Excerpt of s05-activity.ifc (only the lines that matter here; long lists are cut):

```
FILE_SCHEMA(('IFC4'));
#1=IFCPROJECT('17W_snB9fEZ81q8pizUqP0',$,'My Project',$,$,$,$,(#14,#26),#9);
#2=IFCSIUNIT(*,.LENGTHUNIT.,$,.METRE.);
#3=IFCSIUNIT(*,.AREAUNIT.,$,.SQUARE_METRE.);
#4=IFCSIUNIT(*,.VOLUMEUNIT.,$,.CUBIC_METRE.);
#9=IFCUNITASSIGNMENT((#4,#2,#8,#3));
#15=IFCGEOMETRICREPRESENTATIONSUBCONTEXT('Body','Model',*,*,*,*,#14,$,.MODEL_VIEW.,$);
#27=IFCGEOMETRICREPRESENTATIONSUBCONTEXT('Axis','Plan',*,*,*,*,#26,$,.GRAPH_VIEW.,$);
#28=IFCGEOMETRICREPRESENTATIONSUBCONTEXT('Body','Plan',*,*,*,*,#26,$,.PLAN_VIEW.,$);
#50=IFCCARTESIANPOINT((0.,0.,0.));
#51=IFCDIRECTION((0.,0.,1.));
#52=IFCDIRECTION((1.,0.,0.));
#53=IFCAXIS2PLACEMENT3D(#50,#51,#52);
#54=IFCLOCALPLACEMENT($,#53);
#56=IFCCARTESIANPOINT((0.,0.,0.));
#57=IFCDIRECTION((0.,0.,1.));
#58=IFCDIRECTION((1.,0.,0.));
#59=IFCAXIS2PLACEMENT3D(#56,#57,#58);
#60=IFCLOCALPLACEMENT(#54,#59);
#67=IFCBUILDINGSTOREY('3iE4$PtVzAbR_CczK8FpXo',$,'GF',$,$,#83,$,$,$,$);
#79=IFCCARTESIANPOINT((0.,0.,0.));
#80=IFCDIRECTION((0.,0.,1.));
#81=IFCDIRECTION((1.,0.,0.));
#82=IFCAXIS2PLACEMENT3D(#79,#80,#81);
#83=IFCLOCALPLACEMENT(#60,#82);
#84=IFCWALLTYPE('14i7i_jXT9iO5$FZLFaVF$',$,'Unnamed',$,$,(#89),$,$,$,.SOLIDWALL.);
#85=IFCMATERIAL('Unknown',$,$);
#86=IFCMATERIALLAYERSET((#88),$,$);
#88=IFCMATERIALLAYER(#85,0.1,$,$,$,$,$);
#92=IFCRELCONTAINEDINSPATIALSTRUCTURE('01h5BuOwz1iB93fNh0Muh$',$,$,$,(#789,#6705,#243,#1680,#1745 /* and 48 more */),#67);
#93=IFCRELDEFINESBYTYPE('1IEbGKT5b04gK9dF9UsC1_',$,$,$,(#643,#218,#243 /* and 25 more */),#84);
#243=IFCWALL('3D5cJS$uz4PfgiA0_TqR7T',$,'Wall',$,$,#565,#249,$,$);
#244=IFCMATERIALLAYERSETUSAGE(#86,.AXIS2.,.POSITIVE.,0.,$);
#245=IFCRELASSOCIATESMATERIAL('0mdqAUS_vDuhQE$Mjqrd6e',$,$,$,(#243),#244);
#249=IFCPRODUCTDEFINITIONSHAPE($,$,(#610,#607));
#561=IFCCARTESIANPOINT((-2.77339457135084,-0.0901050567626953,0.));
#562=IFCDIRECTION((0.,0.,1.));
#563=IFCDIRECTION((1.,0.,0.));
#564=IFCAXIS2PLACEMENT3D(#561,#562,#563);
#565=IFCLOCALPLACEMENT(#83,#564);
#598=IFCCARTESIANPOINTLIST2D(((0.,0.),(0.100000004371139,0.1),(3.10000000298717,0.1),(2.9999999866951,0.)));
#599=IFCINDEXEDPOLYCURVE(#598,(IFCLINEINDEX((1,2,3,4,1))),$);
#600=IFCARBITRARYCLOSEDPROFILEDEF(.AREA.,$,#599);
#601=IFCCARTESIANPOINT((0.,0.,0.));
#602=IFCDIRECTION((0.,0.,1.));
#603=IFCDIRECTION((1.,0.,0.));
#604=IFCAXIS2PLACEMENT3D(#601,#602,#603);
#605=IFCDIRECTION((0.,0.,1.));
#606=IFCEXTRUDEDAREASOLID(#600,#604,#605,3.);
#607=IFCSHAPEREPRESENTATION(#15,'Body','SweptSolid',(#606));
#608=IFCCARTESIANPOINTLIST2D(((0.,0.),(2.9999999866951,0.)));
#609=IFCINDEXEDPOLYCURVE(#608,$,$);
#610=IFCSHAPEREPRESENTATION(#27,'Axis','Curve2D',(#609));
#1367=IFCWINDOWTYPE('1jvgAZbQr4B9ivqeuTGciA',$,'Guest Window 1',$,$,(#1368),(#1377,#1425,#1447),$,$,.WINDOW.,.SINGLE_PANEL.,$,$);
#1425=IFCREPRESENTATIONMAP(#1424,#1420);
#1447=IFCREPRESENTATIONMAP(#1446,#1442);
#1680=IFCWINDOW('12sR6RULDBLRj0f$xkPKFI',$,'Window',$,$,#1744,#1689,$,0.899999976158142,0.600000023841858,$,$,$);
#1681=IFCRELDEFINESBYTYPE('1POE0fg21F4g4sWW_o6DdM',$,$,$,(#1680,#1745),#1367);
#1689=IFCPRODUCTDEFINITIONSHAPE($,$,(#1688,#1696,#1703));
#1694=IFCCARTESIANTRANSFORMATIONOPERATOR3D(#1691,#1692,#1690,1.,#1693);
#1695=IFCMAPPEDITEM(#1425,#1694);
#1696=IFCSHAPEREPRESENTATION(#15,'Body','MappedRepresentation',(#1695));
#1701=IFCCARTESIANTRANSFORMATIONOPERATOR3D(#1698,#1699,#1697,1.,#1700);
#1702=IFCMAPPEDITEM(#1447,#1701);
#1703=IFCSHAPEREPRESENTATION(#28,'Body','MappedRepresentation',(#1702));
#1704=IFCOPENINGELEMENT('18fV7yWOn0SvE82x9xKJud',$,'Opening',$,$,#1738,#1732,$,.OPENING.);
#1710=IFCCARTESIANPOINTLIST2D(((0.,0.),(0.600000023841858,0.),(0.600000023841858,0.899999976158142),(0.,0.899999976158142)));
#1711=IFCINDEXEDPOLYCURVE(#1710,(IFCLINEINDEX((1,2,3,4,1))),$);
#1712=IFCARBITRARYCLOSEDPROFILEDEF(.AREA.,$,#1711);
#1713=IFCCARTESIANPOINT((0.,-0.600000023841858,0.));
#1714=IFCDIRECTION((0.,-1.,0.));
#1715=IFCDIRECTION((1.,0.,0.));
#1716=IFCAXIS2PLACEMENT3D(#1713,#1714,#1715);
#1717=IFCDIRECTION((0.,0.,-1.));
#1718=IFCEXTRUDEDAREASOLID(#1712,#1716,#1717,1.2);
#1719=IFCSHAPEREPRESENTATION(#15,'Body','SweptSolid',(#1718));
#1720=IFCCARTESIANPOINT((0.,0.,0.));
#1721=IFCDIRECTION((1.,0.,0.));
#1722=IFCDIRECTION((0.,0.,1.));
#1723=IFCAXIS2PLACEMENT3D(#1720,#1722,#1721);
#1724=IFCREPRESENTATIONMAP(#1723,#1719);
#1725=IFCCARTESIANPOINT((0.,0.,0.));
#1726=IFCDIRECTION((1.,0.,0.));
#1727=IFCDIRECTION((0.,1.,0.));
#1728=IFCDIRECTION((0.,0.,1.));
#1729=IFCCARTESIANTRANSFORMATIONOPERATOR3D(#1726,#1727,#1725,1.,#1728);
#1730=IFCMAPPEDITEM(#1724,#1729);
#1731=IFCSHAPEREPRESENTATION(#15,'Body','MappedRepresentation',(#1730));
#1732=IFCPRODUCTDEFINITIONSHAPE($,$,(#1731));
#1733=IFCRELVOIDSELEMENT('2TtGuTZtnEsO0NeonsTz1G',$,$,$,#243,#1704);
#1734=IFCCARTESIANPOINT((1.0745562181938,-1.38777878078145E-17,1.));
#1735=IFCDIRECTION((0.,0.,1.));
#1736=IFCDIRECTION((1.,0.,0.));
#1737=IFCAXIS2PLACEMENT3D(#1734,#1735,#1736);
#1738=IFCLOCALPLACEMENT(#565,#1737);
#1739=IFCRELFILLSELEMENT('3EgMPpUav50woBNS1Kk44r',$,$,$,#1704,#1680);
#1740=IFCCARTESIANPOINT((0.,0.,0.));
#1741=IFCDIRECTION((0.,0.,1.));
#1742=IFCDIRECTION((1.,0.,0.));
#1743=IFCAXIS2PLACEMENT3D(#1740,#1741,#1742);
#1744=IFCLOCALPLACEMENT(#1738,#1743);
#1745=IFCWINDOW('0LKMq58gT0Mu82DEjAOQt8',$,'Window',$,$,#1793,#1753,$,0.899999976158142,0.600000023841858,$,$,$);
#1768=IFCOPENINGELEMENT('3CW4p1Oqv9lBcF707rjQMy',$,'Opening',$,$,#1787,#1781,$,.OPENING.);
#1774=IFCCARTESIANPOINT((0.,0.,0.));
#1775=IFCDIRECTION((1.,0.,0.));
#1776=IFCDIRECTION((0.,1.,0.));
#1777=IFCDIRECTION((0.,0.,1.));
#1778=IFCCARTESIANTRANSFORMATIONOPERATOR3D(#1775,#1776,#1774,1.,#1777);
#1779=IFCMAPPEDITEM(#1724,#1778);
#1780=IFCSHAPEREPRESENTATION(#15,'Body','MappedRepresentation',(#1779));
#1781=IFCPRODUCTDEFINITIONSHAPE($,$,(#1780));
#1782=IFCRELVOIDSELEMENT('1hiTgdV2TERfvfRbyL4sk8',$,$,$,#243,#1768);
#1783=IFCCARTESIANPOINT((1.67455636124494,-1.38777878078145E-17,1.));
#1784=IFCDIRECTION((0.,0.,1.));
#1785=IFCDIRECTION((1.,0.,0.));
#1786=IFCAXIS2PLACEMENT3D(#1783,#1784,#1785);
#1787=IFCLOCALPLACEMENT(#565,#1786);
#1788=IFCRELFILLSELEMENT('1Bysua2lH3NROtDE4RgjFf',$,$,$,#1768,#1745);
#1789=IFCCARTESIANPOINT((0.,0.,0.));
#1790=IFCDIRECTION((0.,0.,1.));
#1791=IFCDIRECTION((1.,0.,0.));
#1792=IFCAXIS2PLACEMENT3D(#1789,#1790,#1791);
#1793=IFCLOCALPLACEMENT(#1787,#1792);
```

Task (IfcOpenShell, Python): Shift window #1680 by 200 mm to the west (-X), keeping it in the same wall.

```python
import ifcopenshell
import ifcopenshell.api.geometry
import ifcopenshell.util.placement
import ifcopenshell.util.unit

model = ifcopenshell.open("s05-activity.ifc")
unit_scale = ifcopenshell.util.unit.calculate_unit_scale(model)

window = model.by_guid("12sR6RULDBLRj0f$xkPKFI")
opening = window.FillsVoids[0].RelatingOpeningElement
wall = opening.VoidsElements[0].RelatingBuildingElement

wall_matrix = ifcopenshell.util.placement.get_local_placement(wall.ObjectPlacement)
shift = wall_matrix[:3, 0] * -0.2 / unit_scale
before = ifcopenshell.util.placement.get_local_placement(window.ObjectPlacement)[:3, 3].copy()

# The window is placed relative to its opening, so it follows when the opening moves.
matrix = ifcopenshell.util.placement.get_local_placement(opening.ObjectPlacement)
matrix[:3, 3] += shift
ifcopenshell.api.geometry.edit_object_placement(
    model, product=opening, matrix=matrix, is_si=False, should_transform_children=True
)

after = ifcopenshell.util.placement.get_local_placement(window.ObjectPlacement)[:3, 3]
print("window moved by", (after - before).round(3) + 0.0)

model.write("s05-activity-out.ifc")
```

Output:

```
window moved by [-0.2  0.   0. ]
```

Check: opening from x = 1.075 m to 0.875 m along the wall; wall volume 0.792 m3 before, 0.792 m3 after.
